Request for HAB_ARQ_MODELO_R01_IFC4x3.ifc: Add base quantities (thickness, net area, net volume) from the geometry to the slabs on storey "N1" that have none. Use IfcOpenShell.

First a look at what the model holds.

```python
import ifcopenshell
import ifcopenshell.util.element
import ifcopenshell.util.unit

model = ifcopenshell.open("HAB_ARQ_MODELO_R01_IFC4x3.ifc")
print(model.schema)
for unit_type in ("LENGTHUNIT", "AREAUNIT", "VOLUMEUNIT"):
    print(unit_type, ifcopenshell.util.unit.calculate_unit_scale(model, unit_type))
storey = next(s for s in model.by_type("IfcBuildingStorey") if s.Name == "N1")
slabs = [e for e in ifcopenshell.util.element.get_decomposition(storey) if e.is_a("IfcSlab")]
for e in sorted(slabs, key=lambda e: e.id()):
    print(e.id(), e.is_a(), e.Name, list(ifcopenshell.util.element.get_psets(e, qtos_only=True)), sep=" | ")
```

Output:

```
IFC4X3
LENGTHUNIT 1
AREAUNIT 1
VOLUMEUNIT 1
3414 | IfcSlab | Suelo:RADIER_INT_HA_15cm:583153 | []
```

```python
import ifcopenshell
import ifcopenshell.api.pset
import ifcopenshell.geom
import ifcopenshell.util.element
import ifcopenshell.util.shape
import ifcopenshell.util.unit

model = ifcopenshell.open("HAB_ARQ_MODELO_R01_IFC4x3.ifc")
unit_scale = ifcopenshell.util.unit.calculate_unit_scale(model)
area_scale = ifcopenshell.util.unit.calculate_unit_scale(model, "AREAUNIT")
volume_scale = ifcopenshell.util.unit.calculate_unit_scale(model, "VOLUMEUNIT")
settings = ifcopenshell.geom.settings()

storey = next(s for s in model.by_type("IfcBuildingStorey") if s.Name == "N1")
slabs = [e for e in ifcopenshell.util.element.get_decomposition(storey) if e.is_a("IfcSlab")]

for e in sorted(slabs, key=lambda e: e.id()):
    if ifcopenshell.util.element.get_psets(e, qtos_only=True, should_inherit=False):
        continue
    # Geometry comes back in metres, in the element's own axes.
    shape = ifcopenshell.geom.create_shape(settings, e)
    values = {
        "Width": ifcopenshell.util.shape.get_z(shape.geometry) / unit_scale,
        "NetArea": ifcopenshell.util.shape.get_footprint_area(shape.geometry) / area_scale,
        "NetVolume": ifcopenshell.util.shape.get_volume(shape.geometry) / volume_scale,
    }
    qto = ifcopenshell.api.pset.add_qto(model, product=e, name="Qto_SlabBaseQuantities")
    ifcopenshell.api.pset.edit_qto(model, qto=qto, properties=values)
    print(e.id(), {k: round(v, 3) for k, v in values.items()})

model.write("HAB_ARQ_MODELO_R01_IFC4x3_edited.ifc")
```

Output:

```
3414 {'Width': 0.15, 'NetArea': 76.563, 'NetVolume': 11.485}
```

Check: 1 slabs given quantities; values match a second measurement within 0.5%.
